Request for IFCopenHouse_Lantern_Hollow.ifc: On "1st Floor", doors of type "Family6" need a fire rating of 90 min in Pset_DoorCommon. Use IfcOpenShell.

First a look at what the model holds.

```python
import ifcopenshell
import ifcopenshell.util.element

model = ifcopenshell.open("IFCopenHouse_Lantern_Hollow.ifc")
print(model.schema)
storey = next(s for s in model.by_type("IfcBuildingStorey") if s.Name == "1st Floor")
doors = [e for e in ifcopenshell.util.element.get_decomposition(storey) if e.is_a("IfcDoor")]
seen = {}
for e in doors:
    element_type = ifcopenshell.util.element.get_type(e)
    key = (element_type.Name if element_type != e and element_type else None, ifcopenshell.util.element.get_pset(e, "Pset_DoorCommon", "FireRating"))
    seen[key] = seen.get(key, 0) + 1
for (name, value), count in sorted(seen.items(), key=str):
    print(count, "x", name, "|", value)
```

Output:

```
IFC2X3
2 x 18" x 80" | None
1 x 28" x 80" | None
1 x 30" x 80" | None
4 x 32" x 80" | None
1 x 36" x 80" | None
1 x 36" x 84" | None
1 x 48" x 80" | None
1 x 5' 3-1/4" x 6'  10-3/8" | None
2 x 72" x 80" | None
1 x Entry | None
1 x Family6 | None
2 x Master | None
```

```python
import ifcopenshell
import ifcopenshell.api.pset
import ifcopenshell.util.element

model = ifcopenshell.open("IFCopenHouse_Lantern_Hollow.ifc")

storey = next(s for s in model.by_type("IfcBuildingStorey") if s.Name == "1st Floor")
doors = [e for e in ifcopenshell.util.element.get_decomposition(storey) if e.is_a("IfcDoor")]

count = 0
for e in doors:
    element_type = ifcopenshell.util.element.get_type(e)
    if element_type in (None, e) or element_type.Name != "Family6":
        continue
    # add_pset returns the element's existing set when there is one.
    pset = ifcopenshell.api.pset.add_pset(model, product=e, name="Pset_DoorCommon")
    ifcopenshell.api.pset.edit_pset(model, pset=pset, properties={"FireRating": "90 min"})
    count += 1

print(count, "doors updated")

model.write("IFCopenHouse_Lantern_Hollow-out.ifc")
```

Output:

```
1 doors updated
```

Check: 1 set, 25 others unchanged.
